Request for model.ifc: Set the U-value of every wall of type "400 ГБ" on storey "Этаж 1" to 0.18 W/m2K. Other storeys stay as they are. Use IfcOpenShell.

First a look at what the model holds.

```python
import ifcopenshell
import ifcopenshell.util.element

model = ifcopenshell.open("model.ifc")
print(model.schema)
storey = next(s for s in model.by_type("IfcBuildingStorey") if s.Name == "Этаж 1")
walls = [e for e in ifcopenshell.util.element.get_decomposition(storey) if e.is_a("IfcWall")]
seen = {}
for e in walls:
    element_type = ifcopenshell.util.element.get_type(e)
    key = (element_type.Name if element_type != e and element_type else None, ifcopenshell.util.element.get_pset(e, "Pset_WallCommon", "ThermalTransmittance"))
    seen[key] = seen.get(key, 0) + 1
for (name, value), count in sorted(seen.items(), key=str):
    print(count, "x", name, "|", value)
```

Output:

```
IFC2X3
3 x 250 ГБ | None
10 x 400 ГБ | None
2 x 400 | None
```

```python
import ifcopenshell
import ifcopenshell.api.pset
import ifcopenshell.util.element

model = ifcopenshell.open("model.ifc")

storey = next(s for s in model.by_type("IfcBuildingStorey") if s.Name == "Этаж 1")
walls = [e for e in ifcopenshell.util.element.get_decomposition(storey) if e.is_a("IfcWall")]

count = 0
for e in walls:
    element_type = ifcopenshell.util.element.get_type(e)
    if element_type in (None, e) or element_type.Name != "400 ГБ":
        continue
    # add_pset returns the element's existing set when there is one.
    pset = ifcopenshell.api.pset.add_pset(model, product=e, name="Pset_WallCommon")
    ifcopenshell.api.pset.edit_pset(model, pset=pset, properties={"ThermalTransmittance": 0.18})
    count += 1

print(count, "walls updated")

model.write("model_rev.ifc")
```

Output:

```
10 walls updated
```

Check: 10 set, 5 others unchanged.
